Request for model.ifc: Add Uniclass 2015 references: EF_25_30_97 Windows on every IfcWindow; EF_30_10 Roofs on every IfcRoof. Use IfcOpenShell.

First a look at what the model holds.

```python
import ifcopenshell

model = ifcopenshell.open("model.ifc")
print(model.schema)
print("classifications:", [c.Name for c in model.by_type("IfcClassification")])
for ifc_class in ("IfcDoor", "IfcRoof", "IfcStair", "IfcWall", "IfcWindow"):
    print(ifc_class, len(model.by_type(ifc_class)))
```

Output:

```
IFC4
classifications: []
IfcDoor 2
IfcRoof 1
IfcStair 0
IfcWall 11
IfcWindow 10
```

```python
import ifcopenshell
import ifcopenshell.api.classification

model = ifcopenshell.open("model.ifc")

system = ifcopenshell.api.classification.add_classification(model, classification="Uniclass 2015")

codes = {
    "IfcWindow": ("EF_25_30_97", "Windows"),
    "IfcRoof": ("EF_30_10", "Roofs"),
}
for ifc_class, (code, name) in codes.items():
    products = model.by_type(ifc_class)
    ifcopenshell.api.classification.add_reference(
        model, products=products, classification=system, identification=code, name=name
    )
    print(code, len(products))

model.write("model_v2.ifc")
```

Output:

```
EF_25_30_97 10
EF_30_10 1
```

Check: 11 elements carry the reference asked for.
